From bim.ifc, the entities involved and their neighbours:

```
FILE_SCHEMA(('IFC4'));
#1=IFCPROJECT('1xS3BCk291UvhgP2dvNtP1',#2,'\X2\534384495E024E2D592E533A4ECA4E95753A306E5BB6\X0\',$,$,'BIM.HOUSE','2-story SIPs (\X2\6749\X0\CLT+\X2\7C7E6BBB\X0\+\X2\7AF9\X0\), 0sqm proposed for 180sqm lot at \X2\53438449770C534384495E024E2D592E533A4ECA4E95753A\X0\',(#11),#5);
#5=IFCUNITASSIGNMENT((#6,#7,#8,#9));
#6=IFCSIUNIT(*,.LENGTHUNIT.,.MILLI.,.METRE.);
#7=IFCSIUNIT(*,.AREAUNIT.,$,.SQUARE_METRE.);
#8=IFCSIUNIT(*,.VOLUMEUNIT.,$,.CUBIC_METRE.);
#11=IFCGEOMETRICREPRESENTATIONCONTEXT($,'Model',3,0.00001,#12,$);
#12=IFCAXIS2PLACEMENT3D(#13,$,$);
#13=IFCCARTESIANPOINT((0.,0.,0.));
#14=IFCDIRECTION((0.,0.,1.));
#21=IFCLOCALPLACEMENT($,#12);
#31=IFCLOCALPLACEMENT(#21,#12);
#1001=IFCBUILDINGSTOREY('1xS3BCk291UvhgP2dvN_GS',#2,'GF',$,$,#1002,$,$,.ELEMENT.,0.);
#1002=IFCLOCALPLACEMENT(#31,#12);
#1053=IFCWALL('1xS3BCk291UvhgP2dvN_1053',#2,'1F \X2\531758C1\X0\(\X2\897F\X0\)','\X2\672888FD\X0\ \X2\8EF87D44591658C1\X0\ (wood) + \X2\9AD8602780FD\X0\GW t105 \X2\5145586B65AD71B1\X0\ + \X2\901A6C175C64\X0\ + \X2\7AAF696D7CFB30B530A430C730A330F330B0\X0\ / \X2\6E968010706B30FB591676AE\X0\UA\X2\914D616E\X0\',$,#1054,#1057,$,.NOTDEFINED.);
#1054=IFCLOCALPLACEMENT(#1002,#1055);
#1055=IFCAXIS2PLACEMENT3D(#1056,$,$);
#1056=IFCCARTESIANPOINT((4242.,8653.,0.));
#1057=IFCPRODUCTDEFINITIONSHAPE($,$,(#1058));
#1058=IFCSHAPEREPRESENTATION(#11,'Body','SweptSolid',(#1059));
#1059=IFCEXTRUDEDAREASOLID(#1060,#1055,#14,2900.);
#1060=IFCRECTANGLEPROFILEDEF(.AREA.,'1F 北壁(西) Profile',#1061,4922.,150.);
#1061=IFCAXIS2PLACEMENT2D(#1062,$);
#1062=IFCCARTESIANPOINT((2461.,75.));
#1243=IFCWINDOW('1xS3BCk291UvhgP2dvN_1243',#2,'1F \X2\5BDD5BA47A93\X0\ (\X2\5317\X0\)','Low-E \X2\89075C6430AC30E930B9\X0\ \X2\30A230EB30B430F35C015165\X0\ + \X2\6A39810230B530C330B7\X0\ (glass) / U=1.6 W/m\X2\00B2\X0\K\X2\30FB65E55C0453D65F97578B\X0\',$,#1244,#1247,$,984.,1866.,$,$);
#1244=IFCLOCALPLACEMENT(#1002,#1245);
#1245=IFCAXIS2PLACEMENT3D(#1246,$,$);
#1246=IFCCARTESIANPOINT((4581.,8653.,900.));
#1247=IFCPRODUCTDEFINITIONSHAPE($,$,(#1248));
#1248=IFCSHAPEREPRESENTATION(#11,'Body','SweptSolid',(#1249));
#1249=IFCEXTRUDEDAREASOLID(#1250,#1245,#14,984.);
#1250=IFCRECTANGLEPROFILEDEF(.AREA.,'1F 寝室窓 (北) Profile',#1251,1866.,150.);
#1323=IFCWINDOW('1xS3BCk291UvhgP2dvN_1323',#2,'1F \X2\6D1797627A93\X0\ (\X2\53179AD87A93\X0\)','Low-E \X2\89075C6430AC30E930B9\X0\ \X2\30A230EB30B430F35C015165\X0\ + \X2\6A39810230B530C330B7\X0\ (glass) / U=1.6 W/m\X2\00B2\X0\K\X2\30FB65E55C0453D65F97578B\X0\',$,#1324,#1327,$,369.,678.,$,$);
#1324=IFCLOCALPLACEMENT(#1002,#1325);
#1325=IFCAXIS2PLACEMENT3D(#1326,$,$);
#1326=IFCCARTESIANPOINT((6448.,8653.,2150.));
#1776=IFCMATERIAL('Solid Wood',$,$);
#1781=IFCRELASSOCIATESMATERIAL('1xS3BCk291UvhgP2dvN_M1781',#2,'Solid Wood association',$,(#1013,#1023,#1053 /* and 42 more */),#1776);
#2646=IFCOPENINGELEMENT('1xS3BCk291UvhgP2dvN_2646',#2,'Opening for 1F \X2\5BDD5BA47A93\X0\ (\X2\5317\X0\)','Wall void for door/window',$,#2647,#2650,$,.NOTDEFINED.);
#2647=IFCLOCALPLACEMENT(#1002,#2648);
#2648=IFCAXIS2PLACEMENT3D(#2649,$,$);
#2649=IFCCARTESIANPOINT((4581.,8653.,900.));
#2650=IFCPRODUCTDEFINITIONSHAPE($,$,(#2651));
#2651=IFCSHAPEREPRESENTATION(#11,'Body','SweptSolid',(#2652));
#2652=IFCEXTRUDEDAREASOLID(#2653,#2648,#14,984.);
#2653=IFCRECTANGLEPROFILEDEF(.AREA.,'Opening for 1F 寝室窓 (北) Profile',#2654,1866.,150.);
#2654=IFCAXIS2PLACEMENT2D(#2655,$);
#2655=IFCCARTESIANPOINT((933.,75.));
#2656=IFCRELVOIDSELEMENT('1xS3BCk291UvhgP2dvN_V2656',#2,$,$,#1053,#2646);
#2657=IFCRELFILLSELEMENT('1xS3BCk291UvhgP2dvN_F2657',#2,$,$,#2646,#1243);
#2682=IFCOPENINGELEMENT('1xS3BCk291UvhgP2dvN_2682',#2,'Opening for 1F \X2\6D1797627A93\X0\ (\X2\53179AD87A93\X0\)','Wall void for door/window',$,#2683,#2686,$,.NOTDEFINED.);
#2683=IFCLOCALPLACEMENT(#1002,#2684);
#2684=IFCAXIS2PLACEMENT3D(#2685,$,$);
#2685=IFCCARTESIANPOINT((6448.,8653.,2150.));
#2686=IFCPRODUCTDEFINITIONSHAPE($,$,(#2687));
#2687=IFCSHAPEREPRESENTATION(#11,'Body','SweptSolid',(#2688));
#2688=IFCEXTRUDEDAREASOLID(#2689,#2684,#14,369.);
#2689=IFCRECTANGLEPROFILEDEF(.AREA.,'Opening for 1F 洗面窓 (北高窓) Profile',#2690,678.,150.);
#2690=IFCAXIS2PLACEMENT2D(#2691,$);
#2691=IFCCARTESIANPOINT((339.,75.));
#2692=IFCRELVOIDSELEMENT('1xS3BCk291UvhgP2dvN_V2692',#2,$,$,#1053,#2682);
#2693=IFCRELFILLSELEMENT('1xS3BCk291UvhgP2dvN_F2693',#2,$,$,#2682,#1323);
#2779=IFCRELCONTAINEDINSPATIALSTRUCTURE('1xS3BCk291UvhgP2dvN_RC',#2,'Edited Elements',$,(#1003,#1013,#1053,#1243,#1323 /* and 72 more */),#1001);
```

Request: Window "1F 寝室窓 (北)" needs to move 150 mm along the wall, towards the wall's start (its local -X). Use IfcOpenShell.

```python
import ifcopenshell
import ifcopenshell.api.geometry
import ifcopenshell.util.placement
import ifcopenshell.util.unit

model = ifcopenshell.open("bim.ifc")
unit_scale = ifcopenshell.util.unit.calculate_unit_scale(model)

window = model.by_guid("1xS3BCk291UvhgP2dvN_1243")
opening = window.FillsVoids[0].RelatingOpeningElement
wall = opening.VoidsElements[0].RelatingBuildingElement

wall_matrix = ifcopenshell.util.placement.get_local_placement(wall.ObjectPlacement)
shift = wall_matrix[:3, 0] * -0.15 / unit_scale
before = ifcopenshell.util.placement.get_local_placement(window.ObjectPlacement)[:3, 3].copy()

# The window is not placed relative to its opening, so move both.
for product in (opening, window):
    matrix = ifcopenshell.util.placement.get_local_placement(product.ObjectPlacement)
    matrix[:3, 3] += shift
    ifcopenshell.api.geometry.edit_object_placement(model, product=product, matrix=matrix, is_si=False)

after = ifcopenshell.util.placement.get_local_placement(window.ObjectPlacement)[:3, 3]
print("window moved by", (after - before).round(3) + 0.0)

model.write("bim_rev.ifc")
```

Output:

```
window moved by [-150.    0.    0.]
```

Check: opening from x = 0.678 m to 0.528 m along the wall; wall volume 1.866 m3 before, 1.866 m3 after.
